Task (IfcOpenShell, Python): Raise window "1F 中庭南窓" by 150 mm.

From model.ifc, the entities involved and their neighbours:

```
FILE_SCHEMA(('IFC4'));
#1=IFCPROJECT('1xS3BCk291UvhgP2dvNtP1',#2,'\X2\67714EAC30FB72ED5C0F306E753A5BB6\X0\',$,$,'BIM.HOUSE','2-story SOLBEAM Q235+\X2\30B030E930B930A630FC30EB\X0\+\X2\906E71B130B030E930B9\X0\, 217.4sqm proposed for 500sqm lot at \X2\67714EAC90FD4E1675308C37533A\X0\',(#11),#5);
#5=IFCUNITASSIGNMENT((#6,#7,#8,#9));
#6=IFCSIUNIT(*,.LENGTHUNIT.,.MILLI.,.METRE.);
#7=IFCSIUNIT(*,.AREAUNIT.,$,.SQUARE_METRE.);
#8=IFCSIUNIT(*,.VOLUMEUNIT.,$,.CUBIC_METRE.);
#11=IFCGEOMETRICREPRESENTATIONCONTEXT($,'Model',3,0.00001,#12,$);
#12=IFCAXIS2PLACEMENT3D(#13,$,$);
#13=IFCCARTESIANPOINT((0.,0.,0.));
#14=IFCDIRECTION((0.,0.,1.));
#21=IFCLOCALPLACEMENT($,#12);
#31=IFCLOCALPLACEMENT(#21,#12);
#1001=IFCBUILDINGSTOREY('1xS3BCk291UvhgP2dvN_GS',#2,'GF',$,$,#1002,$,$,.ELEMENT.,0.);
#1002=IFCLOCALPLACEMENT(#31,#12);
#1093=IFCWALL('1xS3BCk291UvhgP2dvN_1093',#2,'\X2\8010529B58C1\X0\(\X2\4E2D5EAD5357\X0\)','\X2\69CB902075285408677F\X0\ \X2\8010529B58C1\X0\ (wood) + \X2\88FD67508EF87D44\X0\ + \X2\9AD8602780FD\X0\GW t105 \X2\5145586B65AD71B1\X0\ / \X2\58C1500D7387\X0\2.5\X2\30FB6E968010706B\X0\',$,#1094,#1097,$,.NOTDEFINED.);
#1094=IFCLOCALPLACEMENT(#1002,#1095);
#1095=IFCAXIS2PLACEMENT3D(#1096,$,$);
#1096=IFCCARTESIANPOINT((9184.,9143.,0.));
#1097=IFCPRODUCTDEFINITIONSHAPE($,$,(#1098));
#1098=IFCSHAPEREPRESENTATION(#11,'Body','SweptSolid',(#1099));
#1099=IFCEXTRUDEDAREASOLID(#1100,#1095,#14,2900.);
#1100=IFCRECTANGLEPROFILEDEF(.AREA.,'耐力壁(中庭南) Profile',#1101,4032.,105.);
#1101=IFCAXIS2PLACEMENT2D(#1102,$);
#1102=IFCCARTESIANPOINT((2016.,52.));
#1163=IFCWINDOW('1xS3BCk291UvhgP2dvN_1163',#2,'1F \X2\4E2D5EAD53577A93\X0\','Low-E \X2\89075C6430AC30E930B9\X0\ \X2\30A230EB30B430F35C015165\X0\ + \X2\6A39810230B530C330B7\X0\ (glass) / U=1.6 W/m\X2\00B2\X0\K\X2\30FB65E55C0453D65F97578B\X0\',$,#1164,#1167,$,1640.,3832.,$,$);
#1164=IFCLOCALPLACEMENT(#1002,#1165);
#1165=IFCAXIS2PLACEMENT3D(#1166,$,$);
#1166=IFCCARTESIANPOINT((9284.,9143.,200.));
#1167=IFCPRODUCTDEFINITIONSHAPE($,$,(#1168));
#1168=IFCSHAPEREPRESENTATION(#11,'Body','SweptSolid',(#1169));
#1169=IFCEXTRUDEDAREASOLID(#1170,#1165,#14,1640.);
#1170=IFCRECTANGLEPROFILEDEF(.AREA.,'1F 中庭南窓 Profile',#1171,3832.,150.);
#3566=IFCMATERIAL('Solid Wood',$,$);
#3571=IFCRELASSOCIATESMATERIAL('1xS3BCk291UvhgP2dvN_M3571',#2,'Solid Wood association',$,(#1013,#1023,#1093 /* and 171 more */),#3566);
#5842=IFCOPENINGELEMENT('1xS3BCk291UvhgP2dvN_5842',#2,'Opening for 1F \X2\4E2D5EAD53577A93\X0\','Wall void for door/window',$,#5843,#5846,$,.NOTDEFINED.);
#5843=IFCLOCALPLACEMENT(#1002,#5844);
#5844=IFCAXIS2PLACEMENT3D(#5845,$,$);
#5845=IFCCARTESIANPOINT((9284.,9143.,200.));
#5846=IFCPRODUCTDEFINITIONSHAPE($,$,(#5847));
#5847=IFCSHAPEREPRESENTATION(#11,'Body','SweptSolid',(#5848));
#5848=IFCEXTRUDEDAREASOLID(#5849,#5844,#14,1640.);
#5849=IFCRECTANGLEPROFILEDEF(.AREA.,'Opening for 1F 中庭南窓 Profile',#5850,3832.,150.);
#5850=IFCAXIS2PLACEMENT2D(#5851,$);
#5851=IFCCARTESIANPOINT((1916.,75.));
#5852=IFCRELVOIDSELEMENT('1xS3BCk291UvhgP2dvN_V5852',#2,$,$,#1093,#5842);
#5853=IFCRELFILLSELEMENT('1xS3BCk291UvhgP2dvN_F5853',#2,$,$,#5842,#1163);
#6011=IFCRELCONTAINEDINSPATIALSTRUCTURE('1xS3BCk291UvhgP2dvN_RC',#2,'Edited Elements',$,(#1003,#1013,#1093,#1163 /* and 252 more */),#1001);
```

```python
import numpy as np
import ifcopenshell
import ifcopenshell.api.geometry
import ifcopenshell.util.placement
import ifcopenshell.util.unit

model = ifcopenshell.open("model.ifc")
unit_scale = ifcopenshell.util.unit.calculate_unit_scale(model)

window = model.by_id(1163)
opening = window.FillsVoids[0].RelatingOpeningElement
dz = 0.15 / unit_scale

shift = np.array([0.0, 0.0, dz])
# The window is not placed relative to its opening, so move both.
for product in (opening, window):
    matrix = ifcopenshell.util.placement.get_local_placement(product.ObjectPlacement)
    matrix[:3, 3] += shift
    ifcopenshell.api.geometry.edit_object_placement(model, product=product, matrix=matrix, is_si=False)

print(f"moved by {dz * unit_scale:+.3f} m")

model.write("model-out.ifc")
```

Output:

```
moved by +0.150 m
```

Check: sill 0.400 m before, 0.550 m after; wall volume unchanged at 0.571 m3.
